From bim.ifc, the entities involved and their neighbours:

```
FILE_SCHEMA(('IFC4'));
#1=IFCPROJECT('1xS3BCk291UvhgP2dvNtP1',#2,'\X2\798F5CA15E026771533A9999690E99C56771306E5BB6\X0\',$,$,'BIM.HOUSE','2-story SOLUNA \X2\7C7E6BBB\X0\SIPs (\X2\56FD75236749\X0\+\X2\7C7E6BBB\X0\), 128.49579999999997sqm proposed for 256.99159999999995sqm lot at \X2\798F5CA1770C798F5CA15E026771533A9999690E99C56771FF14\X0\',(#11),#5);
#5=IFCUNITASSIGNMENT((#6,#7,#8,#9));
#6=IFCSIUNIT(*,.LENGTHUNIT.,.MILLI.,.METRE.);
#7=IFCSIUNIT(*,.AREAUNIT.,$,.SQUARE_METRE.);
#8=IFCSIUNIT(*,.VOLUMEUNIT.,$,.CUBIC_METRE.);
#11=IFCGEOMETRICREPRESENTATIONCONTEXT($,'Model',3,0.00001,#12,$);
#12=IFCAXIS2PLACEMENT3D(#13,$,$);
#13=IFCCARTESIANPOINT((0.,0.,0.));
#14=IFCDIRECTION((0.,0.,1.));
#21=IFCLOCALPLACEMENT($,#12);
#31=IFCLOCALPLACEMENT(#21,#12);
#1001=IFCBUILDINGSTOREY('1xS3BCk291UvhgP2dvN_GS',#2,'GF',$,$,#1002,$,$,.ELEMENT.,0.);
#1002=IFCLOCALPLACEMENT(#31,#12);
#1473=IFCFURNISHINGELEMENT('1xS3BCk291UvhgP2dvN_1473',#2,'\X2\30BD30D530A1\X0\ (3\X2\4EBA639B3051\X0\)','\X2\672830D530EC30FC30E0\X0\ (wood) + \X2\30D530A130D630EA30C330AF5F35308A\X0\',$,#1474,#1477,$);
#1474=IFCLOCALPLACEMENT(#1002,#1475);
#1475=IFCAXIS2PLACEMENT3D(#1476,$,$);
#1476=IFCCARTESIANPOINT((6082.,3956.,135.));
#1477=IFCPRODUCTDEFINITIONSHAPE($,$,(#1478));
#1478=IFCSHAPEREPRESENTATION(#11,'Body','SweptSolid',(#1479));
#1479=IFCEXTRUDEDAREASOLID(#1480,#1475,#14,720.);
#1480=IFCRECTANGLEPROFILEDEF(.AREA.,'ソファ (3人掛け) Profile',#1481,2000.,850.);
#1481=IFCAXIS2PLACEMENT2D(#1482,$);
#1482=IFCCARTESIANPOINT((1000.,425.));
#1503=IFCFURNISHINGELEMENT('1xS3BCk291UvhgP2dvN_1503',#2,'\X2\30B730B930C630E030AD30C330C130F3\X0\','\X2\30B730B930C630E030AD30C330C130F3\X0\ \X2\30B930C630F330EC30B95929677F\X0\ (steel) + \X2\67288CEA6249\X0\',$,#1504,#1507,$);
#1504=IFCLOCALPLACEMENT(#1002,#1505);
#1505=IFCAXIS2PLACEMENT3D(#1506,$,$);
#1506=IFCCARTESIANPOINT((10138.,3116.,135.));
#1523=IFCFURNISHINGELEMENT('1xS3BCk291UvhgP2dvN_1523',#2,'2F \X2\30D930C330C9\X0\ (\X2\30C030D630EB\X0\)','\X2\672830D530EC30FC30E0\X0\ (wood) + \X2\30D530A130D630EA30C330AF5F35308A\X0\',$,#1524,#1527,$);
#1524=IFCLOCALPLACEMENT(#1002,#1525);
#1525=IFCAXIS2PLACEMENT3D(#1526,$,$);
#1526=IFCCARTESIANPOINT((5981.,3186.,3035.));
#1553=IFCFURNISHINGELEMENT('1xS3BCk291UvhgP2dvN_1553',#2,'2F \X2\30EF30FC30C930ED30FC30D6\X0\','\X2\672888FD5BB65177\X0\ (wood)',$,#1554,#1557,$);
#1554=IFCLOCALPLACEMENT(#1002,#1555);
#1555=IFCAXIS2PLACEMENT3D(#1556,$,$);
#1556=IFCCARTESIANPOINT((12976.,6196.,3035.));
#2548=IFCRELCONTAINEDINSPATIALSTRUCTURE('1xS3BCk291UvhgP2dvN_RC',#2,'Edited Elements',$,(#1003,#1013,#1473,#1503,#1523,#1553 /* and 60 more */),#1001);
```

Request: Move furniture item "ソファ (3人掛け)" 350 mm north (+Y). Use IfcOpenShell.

```python
import ifcopenshell
import ifcopenshell.api.geometry
import ifcopenshell.util.placement
import ifcopenshell.util.unit

model = ifcopenshell.open("bim.ifc")
unit_scale = ifcopenshell.util.unit.calculate_unit_scale(model)

item = model.by_guid("1xS3BCk291UvhgP2dvN_1473")
matrix = ifcopenshell.util.placement.get_local_placement(item.ObjectPlacement)
matrix[1, 3] += 0.35 / unit_scale
ifcopenshell.api.geometry.edit_object_placement(model, product=item, matrix=matrix, is_si=False)

print(ifcopenshell.util.placement.get_local_placement(item.ObjectPlacement).round(3) + 0.0)

model.write("bim_updated.ifc")
```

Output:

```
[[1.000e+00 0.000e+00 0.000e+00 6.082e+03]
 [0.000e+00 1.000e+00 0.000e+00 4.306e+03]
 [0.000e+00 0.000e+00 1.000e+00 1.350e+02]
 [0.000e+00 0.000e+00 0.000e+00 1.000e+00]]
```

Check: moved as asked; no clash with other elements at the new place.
